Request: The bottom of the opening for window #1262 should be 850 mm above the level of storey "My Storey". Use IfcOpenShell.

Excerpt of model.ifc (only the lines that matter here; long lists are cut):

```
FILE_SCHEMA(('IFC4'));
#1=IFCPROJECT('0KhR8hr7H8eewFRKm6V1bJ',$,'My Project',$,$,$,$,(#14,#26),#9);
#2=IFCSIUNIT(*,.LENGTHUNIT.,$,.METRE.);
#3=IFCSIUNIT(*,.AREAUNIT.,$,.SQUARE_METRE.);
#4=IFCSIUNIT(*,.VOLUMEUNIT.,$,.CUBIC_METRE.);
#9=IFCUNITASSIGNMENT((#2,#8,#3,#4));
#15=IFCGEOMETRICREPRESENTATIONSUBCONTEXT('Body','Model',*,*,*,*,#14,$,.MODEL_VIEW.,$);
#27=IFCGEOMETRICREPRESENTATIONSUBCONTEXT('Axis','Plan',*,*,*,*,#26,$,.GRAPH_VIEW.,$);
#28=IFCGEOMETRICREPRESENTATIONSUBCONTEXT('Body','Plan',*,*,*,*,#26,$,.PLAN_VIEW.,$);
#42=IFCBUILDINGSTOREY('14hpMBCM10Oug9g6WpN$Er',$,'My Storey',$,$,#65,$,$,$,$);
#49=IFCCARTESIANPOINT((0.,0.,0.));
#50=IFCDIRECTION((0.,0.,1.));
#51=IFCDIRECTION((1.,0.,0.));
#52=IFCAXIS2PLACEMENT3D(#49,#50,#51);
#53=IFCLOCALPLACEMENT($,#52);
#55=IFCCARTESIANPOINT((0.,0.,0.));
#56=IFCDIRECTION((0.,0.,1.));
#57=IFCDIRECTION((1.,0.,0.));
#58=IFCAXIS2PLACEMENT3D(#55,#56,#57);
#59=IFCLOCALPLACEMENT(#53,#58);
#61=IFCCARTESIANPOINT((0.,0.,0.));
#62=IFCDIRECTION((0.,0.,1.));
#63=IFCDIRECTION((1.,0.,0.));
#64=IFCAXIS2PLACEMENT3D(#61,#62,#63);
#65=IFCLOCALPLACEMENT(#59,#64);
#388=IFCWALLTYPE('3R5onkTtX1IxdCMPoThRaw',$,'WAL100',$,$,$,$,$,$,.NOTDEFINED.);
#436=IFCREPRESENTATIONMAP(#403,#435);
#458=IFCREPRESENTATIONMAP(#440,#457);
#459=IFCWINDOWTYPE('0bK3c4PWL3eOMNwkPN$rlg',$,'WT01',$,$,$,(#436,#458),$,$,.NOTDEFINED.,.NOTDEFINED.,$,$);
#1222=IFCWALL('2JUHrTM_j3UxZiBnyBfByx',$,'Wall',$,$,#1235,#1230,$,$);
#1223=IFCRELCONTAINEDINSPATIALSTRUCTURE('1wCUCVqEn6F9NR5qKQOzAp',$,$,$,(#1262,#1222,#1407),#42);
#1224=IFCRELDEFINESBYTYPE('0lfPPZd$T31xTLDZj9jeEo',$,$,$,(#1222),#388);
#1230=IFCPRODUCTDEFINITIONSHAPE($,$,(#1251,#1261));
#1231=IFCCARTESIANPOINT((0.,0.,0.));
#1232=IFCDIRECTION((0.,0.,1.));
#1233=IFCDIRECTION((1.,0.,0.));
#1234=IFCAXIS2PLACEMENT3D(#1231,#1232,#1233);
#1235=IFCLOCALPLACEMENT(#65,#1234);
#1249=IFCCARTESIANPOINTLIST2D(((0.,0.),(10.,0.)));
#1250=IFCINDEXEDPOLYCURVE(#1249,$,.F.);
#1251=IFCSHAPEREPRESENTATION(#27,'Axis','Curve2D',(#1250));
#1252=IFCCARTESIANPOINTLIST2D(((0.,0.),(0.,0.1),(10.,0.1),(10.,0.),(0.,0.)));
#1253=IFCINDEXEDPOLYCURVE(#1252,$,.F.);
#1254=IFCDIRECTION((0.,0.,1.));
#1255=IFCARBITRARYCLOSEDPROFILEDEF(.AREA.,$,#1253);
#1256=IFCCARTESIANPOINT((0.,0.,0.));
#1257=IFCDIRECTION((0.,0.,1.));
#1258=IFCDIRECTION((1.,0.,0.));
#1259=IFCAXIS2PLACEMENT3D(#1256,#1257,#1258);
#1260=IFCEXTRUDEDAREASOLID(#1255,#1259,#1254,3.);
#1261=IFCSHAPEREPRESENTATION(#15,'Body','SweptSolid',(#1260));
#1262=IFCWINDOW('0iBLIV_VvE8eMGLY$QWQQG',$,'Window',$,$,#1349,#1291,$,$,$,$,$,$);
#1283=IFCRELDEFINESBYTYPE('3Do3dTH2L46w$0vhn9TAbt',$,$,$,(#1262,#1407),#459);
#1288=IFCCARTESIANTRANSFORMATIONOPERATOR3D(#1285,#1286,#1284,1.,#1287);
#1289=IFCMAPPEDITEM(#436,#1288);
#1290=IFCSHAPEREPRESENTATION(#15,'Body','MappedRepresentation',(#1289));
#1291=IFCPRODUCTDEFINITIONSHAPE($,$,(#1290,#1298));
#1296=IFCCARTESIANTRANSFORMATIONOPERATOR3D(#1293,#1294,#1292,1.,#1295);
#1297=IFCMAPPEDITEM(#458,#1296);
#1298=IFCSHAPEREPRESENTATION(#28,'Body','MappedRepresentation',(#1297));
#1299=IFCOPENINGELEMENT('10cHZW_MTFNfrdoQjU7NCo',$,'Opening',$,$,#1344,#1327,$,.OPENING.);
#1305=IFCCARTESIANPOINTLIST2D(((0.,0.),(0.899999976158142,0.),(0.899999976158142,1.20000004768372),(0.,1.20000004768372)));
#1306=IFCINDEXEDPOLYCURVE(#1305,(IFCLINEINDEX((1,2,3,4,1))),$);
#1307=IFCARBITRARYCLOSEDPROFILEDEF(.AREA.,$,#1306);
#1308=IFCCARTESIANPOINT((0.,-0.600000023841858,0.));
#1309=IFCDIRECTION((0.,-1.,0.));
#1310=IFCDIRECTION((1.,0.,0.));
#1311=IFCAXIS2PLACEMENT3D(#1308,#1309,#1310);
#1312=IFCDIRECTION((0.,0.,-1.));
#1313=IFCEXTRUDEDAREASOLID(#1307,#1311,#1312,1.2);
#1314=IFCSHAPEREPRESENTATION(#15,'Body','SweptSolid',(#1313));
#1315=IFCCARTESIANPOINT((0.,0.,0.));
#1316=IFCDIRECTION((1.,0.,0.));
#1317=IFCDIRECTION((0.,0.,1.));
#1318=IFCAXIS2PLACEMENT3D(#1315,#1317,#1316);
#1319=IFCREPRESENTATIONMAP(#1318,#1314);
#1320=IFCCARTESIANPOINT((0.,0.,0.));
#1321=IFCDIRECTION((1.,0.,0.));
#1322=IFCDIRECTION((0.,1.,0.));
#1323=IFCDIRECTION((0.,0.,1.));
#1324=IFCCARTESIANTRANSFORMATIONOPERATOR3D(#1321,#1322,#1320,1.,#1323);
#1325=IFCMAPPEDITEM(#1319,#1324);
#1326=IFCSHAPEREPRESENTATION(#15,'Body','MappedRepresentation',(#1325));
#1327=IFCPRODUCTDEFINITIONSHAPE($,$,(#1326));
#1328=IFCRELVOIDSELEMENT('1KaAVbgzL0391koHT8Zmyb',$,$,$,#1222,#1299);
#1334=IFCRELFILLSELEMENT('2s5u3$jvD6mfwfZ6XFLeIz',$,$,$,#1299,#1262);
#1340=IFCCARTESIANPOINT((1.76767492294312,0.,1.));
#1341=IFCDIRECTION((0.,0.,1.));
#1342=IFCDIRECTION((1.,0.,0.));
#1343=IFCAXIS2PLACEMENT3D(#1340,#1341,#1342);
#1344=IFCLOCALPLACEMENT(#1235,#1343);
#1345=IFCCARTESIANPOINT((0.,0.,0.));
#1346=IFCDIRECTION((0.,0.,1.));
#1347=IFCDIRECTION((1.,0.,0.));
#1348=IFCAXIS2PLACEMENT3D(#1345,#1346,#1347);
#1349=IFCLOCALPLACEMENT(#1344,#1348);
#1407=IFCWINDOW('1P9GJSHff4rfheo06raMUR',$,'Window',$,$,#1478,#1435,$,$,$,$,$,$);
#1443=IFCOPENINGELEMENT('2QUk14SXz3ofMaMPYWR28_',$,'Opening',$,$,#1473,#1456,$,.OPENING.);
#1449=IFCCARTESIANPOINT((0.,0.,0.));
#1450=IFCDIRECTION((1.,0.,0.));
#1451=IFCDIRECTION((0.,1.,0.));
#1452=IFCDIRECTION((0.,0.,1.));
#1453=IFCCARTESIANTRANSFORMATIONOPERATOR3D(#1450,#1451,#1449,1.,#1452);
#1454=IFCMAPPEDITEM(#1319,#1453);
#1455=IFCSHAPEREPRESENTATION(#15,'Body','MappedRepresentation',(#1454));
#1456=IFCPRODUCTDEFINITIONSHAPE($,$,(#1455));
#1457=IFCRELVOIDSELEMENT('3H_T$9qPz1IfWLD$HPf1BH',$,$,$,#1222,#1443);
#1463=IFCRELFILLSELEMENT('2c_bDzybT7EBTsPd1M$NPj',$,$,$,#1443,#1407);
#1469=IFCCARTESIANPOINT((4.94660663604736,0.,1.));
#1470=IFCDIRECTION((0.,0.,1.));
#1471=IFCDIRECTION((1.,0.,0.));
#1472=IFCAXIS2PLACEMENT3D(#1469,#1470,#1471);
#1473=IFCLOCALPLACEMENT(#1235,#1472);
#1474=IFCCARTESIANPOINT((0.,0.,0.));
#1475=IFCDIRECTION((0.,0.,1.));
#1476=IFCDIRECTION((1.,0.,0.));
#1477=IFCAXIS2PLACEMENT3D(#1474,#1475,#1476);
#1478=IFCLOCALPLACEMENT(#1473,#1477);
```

```python
import numpy as np
import ifcopenshell
import ifcopenshell.api.geometry
import ifcopenshell.geom
import ifcopenshell.util.element
import ifcopenshell.util.placement
import ifcopenshell.util.shape
import ifcopenshell.util.unit

model = ifcopenshell.open("model.ifc")
unit_scale = ifcopenshell.util.unit.calculate_unit_scale(model)

window = model.by_id(1262)
opening = window.FillsVoids[0].RelatingOpeningElement
storey = ifcopenshell.util.element.get_container(window, ifc_class="IfcBuildingStorey")
level = ifcopenshell.util.placement.get_local_placement(storey.ObjectPlacement)[2, 3]

# The opening's origin need not be at the sill, so measure its lowest point.
shape = ifcopenshell.geom.create_shape(ifcopenshell.geom.settings(), opening)
bottom = ifcopenshell.util.shape.get_shape_bottom_elevation(shape, shape.geometry) / unit_scale
dz = level + 0.85 - bottom

shift = np.array([0.0, 0.0, dz])
# The window is placed relative to its opening, so it follows when the opening moves.
matrix = ifcopenshell.util.placement.get_local_placement(opening.ObjectPlacement)
matrix[:3, 3] += shift
ifcopenshell.api.geometry.edit_object_placement(
    model, product=opening, matrix=matrix, is_si=False, should_transform_children=True
)

print(f"moved by {dz * unit_scale:+.3f} m")

model.write("model_rev.ifc")
```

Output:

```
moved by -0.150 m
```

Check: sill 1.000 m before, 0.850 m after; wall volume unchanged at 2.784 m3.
